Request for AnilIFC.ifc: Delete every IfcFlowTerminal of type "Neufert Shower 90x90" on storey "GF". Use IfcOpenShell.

First a look at what the model holds.

```python
import ifcopenshell
import ifcopenshell.util.element

model = ifcopenshell.open("AnilIFC.ifc")
print(model.schema)
storey = next(s for s in model.by_type("IfcBuildingStorey") if s.Name == "GF")
terminals = [e for e in ifcopenshell.util.element.get_decomposition(storey) if e.is_a("IfcFlowTerminal")]
seen = {}
for e in terminals:
    element_type = ifcopenshell.util.element.get_type(e)
    name = element_type.Name if element_type not in (None, e) else None
    seen[name] = seen.get(name, 0) + 1
for name, count in sorted(seen.items(), key=str):
    print(count, "x", name)
```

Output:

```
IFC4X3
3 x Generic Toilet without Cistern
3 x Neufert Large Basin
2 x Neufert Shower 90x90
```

```python
import ifcopenshell
import ifcopenshell.api.root
import ifcopenshell.util.element

model = ifcopenshell.open("AnilIFC.ifc")

storey = next(s for s in model.by_type("IfcBuildingStorey") if s.Name == "GF")
terminals = [e for e in ifcopenshell.util.element.get_decomposition(storey) if e.is_a("IfcFlowTerminal")]
targets = [e for e in terminals if (t := ifcopenshell.util.element.get_type(e)) not in (None, e) and t.Name == "Neufert Shower 90x90"]

for e in targets:
    ifcopenshell.api.root.remove_product(model, product=e)
print(len(targets), "removed")

model.write("AnilIFC_rev.ifc")
```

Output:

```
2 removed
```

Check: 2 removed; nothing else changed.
